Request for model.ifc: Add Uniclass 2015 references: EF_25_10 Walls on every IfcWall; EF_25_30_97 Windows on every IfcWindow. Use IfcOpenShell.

First a look at what the model holds.

```python
import ifcopenshell

model = ifcopenshell.open("model.ifc")
print(model.schema)
print("classifications:", [c.Name for c in model.by_type("IfcClassification")])
for ifc_class in ("IfcDoor", "IfcRoof", "IfcStair", "IfcWall", "IfcWindow"):
    print(ifc_class, len(model.by_type(ifc_class)))
```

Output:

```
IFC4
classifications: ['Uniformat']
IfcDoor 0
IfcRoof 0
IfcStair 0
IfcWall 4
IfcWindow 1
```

```python
import ifcopenshell
import ifcopenshell.api.classification

model = ifcopenshell.open("model.ifc")

system = ifcopenshell.api.classification.add_classification(model, classification="Uniclass 2015")

codes = {
    "IfcWall": ("EF_25_10", "Walls"),
    "IfcWindow": ("EF_25_30_97", "Windows"),
}
for ifc_class, (code, name) in codes.items():
    products = model.by_type(ifc_class)
    ifcopenshell.api.classification.add_reference(
        model, products=products, classification=system, identification=code, name=name
    )
    print(code, len(products))

model.write("model-out.ifc")
```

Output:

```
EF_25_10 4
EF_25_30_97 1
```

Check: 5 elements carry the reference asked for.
